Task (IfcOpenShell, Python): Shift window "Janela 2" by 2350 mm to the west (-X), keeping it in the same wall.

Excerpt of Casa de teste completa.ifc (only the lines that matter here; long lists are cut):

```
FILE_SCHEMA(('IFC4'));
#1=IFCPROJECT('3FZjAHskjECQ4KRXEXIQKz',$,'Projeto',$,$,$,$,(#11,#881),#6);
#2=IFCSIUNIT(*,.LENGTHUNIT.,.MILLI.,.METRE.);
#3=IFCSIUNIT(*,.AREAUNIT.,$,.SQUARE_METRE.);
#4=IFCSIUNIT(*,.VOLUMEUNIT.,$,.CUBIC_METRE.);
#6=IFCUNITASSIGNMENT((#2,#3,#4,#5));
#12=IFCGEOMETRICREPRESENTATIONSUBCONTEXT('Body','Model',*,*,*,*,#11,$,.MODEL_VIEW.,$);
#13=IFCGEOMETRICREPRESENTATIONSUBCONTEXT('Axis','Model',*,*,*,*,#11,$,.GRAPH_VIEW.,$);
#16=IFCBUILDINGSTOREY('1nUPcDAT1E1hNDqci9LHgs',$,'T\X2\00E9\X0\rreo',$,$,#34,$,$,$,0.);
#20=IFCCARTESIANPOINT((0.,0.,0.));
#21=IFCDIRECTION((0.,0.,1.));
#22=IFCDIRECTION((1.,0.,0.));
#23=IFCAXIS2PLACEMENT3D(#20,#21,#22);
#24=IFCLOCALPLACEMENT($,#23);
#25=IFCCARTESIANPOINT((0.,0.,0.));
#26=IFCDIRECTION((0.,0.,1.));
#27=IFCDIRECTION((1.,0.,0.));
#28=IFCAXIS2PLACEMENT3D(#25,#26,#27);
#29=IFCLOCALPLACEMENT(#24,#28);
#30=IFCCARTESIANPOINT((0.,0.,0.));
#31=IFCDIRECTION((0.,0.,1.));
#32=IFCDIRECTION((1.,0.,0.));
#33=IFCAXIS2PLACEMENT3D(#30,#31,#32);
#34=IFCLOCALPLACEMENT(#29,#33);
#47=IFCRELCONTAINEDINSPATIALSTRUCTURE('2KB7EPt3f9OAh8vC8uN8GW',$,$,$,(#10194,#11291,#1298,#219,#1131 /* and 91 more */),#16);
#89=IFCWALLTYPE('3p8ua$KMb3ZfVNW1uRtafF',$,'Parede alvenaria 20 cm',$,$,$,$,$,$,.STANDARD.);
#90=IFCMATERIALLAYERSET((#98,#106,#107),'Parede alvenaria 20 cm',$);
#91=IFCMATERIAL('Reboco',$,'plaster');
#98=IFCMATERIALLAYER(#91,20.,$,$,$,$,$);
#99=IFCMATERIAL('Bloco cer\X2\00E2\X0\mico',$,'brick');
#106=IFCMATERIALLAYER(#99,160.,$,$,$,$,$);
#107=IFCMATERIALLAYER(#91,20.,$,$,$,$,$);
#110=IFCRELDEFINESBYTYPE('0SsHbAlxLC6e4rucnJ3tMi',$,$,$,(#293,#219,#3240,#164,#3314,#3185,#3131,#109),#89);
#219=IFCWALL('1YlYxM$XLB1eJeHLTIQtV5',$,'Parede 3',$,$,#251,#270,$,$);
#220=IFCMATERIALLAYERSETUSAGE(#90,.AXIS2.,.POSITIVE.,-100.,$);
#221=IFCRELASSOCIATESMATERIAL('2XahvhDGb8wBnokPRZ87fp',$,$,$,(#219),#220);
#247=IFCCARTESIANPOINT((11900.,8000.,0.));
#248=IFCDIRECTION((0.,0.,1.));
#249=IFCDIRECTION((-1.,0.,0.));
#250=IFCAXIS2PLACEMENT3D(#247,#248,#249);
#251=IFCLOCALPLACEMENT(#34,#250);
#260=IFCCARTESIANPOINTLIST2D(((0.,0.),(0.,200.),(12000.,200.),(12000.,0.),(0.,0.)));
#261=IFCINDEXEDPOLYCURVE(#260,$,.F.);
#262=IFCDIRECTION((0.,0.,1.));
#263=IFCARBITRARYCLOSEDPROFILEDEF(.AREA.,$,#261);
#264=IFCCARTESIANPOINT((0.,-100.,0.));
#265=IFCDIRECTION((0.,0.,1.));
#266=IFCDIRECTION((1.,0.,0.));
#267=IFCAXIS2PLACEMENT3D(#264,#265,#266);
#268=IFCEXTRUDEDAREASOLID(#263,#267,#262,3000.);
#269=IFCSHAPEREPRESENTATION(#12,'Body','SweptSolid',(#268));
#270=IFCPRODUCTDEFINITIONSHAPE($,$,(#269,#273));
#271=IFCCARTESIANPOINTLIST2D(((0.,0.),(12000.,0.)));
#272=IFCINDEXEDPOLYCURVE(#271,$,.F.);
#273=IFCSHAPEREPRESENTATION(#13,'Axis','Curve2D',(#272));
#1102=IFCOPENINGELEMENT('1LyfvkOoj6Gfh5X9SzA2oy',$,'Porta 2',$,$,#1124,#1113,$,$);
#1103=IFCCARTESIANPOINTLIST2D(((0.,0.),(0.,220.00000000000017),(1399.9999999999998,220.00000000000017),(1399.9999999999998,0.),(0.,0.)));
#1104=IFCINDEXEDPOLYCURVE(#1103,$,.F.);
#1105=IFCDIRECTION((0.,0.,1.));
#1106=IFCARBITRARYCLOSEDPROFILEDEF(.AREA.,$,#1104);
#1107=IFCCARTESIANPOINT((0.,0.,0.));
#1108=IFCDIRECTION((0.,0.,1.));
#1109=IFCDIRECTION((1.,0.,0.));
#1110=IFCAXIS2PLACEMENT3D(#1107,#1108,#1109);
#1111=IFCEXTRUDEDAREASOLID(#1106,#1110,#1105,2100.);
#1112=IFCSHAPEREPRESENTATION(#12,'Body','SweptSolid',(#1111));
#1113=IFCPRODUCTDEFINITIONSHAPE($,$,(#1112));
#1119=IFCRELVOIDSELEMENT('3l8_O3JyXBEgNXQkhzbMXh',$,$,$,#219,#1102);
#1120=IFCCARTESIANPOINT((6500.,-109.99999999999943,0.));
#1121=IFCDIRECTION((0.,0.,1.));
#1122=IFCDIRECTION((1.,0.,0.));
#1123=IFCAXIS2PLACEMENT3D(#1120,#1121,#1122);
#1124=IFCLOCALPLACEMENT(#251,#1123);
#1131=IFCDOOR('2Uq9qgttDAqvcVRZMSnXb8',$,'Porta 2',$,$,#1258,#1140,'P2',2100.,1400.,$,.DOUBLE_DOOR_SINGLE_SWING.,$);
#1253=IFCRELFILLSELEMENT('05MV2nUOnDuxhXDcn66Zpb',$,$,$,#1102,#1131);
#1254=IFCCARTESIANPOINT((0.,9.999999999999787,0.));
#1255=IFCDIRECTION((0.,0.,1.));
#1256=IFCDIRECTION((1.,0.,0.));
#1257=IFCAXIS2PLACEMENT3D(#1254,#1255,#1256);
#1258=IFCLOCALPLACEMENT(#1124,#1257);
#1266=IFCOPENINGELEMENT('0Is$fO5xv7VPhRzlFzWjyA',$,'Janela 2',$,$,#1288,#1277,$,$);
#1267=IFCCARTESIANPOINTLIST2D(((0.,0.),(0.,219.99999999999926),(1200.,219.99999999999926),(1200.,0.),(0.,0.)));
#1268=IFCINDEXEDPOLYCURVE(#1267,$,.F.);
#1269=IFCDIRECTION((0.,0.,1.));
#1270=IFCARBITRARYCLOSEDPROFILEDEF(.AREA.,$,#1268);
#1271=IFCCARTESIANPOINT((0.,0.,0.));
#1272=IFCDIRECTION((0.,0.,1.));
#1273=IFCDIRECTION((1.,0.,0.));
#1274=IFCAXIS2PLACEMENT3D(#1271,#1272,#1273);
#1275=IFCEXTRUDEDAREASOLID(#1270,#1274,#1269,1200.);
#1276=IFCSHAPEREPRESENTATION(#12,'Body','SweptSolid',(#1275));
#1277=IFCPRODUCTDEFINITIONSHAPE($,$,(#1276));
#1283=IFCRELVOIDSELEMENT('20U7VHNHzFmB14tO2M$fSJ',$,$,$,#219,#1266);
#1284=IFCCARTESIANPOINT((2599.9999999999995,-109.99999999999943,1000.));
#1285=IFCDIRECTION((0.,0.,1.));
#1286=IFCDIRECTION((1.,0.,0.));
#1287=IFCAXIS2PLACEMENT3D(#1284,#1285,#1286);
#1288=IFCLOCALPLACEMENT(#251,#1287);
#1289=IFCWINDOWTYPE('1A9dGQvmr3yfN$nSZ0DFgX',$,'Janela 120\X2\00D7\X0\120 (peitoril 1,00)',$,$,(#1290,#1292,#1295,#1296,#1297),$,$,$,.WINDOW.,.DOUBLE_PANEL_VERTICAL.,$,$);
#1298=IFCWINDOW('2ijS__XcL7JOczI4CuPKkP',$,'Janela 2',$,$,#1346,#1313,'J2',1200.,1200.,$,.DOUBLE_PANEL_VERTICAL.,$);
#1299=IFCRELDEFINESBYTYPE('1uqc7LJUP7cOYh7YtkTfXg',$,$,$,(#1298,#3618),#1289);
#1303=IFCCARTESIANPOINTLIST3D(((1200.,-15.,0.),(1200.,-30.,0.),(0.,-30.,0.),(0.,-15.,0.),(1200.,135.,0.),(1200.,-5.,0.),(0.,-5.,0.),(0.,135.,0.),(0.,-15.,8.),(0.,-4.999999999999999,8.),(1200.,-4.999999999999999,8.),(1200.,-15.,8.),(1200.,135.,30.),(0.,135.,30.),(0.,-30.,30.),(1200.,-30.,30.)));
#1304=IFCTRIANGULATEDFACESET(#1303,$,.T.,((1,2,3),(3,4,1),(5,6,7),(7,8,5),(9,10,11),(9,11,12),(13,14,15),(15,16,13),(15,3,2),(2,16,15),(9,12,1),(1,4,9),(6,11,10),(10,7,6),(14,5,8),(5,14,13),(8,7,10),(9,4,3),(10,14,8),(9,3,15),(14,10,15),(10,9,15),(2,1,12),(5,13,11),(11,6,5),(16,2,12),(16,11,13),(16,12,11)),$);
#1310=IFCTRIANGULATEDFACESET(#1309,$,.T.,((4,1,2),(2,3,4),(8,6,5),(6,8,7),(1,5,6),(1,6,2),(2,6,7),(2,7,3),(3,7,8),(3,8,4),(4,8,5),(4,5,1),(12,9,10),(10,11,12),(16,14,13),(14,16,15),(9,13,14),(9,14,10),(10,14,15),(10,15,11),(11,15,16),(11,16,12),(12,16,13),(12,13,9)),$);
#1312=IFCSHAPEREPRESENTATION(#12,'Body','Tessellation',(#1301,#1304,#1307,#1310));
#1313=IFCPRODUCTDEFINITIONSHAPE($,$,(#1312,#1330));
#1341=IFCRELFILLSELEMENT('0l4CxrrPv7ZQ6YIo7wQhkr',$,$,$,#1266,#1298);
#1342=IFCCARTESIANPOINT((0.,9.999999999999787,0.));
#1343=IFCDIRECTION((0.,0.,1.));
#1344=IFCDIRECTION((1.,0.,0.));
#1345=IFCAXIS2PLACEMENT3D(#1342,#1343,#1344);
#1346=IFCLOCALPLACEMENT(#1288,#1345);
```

```python
import ifcopenshell
import ifcopenshell.api.geometry
import ifcopenshell.util.placement

model = ifcopenshell.open("Casa de teste completa.ifc")

window = model.by_id(1298)
opening = window.FillsVoids[0].RelatingOpeningElement
wall = opening.VoidsElements[0].RelatingBuildingElement

wall_matrix = ifcopenshell.util.placement.get_local_placement(wall.ObjectPlacement)
shift = wall_matrix[:3, 0] * 2350.0
before = ifcopenshell.util.placement.get_local_placement(window.ObjectPlacement)[:3, 3].copy()

# The window is placed relative to its opening, so it follows when the opening moves.
matrix = ifcopenshell.util.placement.get_local_placement(opening.ObjectPlacement)
matrix[:3, 3] += shift
ifcopenshell.api.geometry.edit_object_placement(
    model, product=opening, matrix=matrix, is_si=False, should_transform_children=True
)

after = ifcopenshell.util.placement.get_local_placement(window.ObjectPlacement)[:3, 3]
print("window moved by", (after - before).round(3) + 0.0)

model.write("Casa de teste completa_updated.ifc")
```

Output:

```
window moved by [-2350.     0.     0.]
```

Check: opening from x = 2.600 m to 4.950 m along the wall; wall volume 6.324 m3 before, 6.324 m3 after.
